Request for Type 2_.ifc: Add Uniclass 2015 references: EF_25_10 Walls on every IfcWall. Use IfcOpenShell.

First a look at what the model holds.

```python
import ifcopenshell

model = ifcopenshell.open("Type 2_.ifc")
print(model.schema)
print("classifications:", [c.Name for c in model.by_type("IfcClassification")])
for ifc_class in ("IfcDoor", "IfcRoof", "IfcStair", "IfcWall", "IfcWindow"):
    print(ifc_class, len(model.by_type(ifc_class)))
```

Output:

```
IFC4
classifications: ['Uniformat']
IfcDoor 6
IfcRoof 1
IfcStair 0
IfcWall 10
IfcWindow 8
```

```python
import ifcopenshell
import ifcopenshell.api.classification

model = ifcopenshell.open("Type 2_.ifc")

system = ifcopenshell.api.classification.add_classification(model, classification="Uniclass 2015")

codes = {
    "IfcWall": ("EF_25_10", "Walls"),
}
for ifc_class, (code, name) in codes.items():
    products = model.by_type(ifc_class)
    ifcopenshell.api.classification.add_reference(
        model, products=products, classification=system, identification=code, name=name
    )
    print(code, len(products))

model.write("Type 2__updated.ifc")
```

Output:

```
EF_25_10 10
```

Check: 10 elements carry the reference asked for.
